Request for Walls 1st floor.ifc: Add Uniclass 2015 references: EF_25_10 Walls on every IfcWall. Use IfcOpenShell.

First a look at what the model holds.

```python
import ifcopenshell

model = ifcopenshell.open("Walls 1st floor.ifc")
print(model.schema)
print("classifications:", [c.Name for c in model.by_type("IfcClassification")])
for ifc_class in ("IfcDoor", "IfcRoof", "IfcStair", "IfcWall", "IfcWindow"):
    print(ifc_class, len(model.by_type(ifc_class)))
```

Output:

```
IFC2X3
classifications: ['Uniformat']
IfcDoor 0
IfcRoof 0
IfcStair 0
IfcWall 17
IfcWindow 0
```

```python
import ifcopenshell
import ifcopenshell.api.classification

model = ifcopenshell.open("Walls 1st floor.ifc")

# IFC2X3 requires Source and Edition and has no link from the project to the system.
system = model.create_entity("IfcClassification", Source="NBS", Edition="2015", Name="Uniclass 2015")

codes = {
    "IfcWall": ("EF_25_10", "Walls"),
}
for ifc_class, (code, name) in codes.items():
    products = model.by_type(ifc_class)
    ifcopenshell.api.classification.add_reference(
        model, products=products, classification=system, identification=code, name=name
    )
    print(code, len(products))

model.write("Walls 1st floor_edited.ifc")
```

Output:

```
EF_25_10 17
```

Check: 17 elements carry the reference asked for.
